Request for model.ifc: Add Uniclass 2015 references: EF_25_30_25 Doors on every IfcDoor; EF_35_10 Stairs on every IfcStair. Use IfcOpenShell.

First a look at what the model holds.

```python
import ifcopenshell

model = ifcopenshell.open("model.ifc")
print(model.schema)
print("classifications:", [c.Name for c in model.by_type("IfcClassification")])
for ifc_class in ("IfcDoor", "IfcRoof", "IfcStair", "IfcWall", "IfcWindow"):
    print(ifc_class, len(model.by_type(ifc_class)))
```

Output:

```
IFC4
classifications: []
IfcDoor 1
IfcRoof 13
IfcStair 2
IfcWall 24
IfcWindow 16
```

```python
import ifcopenshell
import ifcopenshell.api.classification

model = ifcopenshell.open("model.ifc")

system = ifcopenshell.api.classification.add_classification(model, classification="Uniclass 2015")

codes = {
    "IfcDoor": ("EF_25_30_25", "Doors"),
    "IfcStair": ("EF_35_10", "Stairs"),
}
for ifc_class, (code, name) in codes.items():
    products = model.by_type(ifc_class)
    ifcopenshell.api.classification.add_reference(
        model, products=products, classification=system, identification=code, name=name
    )
    print(code, len(products))

model.write("model-out.ifc")
```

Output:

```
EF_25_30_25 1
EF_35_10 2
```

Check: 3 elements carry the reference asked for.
